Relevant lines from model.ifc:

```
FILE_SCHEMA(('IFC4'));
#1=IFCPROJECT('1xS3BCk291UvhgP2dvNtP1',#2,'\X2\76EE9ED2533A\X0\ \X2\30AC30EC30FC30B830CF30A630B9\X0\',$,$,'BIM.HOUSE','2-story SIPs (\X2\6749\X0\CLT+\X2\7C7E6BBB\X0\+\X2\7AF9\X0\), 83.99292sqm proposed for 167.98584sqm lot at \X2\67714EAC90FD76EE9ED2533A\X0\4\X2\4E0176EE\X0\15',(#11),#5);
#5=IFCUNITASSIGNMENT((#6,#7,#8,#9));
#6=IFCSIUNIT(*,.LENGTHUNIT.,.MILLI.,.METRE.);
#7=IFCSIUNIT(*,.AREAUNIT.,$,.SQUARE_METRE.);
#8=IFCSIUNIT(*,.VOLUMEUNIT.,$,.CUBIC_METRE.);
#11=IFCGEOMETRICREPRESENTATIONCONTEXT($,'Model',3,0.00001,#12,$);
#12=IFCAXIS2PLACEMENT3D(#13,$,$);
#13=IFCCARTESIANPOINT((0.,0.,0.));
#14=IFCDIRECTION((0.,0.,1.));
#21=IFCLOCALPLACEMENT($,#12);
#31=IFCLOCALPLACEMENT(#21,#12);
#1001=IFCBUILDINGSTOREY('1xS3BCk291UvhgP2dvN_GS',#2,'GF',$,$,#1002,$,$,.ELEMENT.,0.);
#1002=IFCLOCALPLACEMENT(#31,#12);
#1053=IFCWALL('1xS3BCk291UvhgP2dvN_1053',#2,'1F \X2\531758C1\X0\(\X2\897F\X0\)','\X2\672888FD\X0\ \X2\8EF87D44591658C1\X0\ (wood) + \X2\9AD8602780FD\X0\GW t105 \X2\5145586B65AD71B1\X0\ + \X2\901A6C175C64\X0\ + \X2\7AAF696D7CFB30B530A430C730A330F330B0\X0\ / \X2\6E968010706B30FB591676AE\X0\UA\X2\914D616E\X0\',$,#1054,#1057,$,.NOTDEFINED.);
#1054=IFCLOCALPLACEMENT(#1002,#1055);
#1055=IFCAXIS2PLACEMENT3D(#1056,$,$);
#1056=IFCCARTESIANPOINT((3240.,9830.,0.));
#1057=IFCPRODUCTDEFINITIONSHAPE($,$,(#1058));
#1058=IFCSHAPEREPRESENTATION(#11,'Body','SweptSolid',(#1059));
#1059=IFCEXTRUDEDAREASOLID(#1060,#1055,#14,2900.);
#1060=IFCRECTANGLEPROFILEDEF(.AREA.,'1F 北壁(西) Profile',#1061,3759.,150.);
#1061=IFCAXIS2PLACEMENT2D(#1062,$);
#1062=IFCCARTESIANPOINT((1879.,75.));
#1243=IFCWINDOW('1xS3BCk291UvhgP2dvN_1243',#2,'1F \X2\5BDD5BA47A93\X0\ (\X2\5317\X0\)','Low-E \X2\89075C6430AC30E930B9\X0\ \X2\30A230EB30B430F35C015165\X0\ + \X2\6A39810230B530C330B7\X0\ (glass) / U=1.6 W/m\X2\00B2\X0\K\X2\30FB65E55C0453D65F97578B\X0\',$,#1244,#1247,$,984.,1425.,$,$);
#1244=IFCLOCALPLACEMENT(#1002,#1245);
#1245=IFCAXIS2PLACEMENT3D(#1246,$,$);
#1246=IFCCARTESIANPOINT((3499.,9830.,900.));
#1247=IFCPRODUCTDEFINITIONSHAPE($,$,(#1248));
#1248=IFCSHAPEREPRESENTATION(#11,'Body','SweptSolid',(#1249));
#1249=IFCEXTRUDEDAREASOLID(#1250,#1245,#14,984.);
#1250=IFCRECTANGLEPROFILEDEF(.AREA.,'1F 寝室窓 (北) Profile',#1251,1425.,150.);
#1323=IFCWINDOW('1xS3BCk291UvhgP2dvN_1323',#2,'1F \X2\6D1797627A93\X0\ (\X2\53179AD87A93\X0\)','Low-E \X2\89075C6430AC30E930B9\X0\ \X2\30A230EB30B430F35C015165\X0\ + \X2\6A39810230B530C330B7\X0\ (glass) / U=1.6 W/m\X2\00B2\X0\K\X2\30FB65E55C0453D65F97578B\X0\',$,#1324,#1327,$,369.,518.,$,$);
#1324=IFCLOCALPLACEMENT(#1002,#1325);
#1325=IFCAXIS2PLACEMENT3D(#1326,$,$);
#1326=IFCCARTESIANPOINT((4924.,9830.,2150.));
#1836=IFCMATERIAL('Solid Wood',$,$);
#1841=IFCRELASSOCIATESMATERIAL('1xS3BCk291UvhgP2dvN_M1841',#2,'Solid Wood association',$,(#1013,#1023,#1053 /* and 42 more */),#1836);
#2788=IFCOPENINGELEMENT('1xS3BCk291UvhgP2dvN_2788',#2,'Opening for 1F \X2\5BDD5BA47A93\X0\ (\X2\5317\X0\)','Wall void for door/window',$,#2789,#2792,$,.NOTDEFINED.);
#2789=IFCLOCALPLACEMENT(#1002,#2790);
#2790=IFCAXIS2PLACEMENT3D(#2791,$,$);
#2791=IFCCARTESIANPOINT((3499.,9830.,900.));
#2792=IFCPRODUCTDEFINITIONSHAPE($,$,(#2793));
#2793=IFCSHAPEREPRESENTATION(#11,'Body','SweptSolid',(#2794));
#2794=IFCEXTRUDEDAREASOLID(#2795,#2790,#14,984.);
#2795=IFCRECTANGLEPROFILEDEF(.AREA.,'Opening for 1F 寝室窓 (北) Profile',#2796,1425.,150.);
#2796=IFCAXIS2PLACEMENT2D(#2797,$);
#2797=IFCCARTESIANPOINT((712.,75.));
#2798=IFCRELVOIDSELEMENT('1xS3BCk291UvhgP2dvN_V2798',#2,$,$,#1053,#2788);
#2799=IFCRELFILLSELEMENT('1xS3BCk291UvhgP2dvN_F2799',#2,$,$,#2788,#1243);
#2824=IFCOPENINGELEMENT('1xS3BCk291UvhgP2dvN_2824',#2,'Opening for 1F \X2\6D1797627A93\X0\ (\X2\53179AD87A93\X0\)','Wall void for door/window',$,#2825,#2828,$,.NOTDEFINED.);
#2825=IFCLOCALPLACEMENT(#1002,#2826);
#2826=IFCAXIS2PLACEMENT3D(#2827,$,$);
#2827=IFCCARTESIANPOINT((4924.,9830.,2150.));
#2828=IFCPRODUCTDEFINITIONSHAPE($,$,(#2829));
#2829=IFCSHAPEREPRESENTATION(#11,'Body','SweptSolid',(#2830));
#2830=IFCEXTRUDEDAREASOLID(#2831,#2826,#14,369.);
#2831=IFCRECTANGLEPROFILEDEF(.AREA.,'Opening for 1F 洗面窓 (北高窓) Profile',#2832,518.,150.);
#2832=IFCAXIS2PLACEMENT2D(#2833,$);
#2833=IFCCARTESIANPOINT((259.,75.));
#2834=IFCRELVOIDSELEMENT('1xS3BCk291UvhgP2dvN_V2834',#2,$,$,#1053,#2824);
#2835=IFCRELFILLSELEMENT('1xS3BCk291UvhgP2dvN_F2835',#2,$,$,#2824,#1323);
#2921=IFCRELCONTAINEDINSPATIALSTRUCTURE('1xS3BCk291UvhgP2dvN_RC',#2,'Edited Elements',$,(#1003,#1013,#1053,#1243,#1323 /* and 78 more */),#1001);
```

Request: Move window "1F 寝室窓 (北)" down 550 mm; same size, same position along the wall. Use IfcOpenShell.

```python
import numpy as np
import ifcopenshell
import ifcopenshell.api.geometry
import ifcopenshell.util.placement
import ifcopenshell.util.unit

model = ifcopenshell.open("model.ifc")
unit_scale = ifcopenshell.util.unit.calculate_unit_scale(model)

window = model.by_guid("1xS3BCk291UvhgP2dvN_1243")
opening = window.FillsVoids[0].RelatingOpeningElement
dz = -0.55 / unit_scale

shift = np.array([0.0, 0.0, dz])
# The window is not placed relative to its opening, so move both.
for product in (opening, window):
    matrix = ifcopenshell.util.placement.get_local_placement(product.ObjectPlacement)
    matrix[:3, 3] += shift
    ifcopenshell.api.geometry.edit_object_placement(model, product=product, matrix=matrix, is_si=False)

print(f"moved by {dz * unit_scale:+.3f} m")

model.write("model_v2.ifc")
```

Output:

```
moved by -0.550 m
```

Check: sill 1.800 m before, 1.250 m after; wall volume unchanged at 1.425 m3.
